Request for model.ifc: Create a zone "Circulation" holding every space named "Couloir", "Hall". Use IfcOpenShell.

First a look at what the model holds.

```python
import ifcopenshell

model = ifcopenshell.open("model.ifc")
print(model.schema)
seen = {}
for space in model.by_type("IfcSpace"):
    seen[space.LongName] = seen.get(space.LongName, 0) + 1
for name, count in sorted(seen.items(), key=str):
    print(count, "x", name)
print("zones:", [z.Name for z in model.by_type("IfcZone")][:20])
```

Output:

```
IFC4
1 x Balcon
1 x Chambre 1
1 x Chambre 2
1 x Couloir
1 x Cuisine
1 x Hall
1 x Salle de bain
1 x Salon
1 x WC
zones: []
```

```python
import ifcopenshell
import ifcopenshell.api.group
import ifcopenshell.api.root

model = ifcopenshell.open("model.ifc")

names = {"Couloir", "Hall"}
spaces = [s for s in model.by_type("IfcSpace") if s.LongName in names]

zone = ifcopenshell.api.root.create_entity(model, ifc_class="IfcZone", name="Circulation")
ifcopenshell.api.group.assign_group(model, products=spaces, group=zone)
print(len(spaces), "spaces in", zone.Name)

model.write("model_updated.ifc")
```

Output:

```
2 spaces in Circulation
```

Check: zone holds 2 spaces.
